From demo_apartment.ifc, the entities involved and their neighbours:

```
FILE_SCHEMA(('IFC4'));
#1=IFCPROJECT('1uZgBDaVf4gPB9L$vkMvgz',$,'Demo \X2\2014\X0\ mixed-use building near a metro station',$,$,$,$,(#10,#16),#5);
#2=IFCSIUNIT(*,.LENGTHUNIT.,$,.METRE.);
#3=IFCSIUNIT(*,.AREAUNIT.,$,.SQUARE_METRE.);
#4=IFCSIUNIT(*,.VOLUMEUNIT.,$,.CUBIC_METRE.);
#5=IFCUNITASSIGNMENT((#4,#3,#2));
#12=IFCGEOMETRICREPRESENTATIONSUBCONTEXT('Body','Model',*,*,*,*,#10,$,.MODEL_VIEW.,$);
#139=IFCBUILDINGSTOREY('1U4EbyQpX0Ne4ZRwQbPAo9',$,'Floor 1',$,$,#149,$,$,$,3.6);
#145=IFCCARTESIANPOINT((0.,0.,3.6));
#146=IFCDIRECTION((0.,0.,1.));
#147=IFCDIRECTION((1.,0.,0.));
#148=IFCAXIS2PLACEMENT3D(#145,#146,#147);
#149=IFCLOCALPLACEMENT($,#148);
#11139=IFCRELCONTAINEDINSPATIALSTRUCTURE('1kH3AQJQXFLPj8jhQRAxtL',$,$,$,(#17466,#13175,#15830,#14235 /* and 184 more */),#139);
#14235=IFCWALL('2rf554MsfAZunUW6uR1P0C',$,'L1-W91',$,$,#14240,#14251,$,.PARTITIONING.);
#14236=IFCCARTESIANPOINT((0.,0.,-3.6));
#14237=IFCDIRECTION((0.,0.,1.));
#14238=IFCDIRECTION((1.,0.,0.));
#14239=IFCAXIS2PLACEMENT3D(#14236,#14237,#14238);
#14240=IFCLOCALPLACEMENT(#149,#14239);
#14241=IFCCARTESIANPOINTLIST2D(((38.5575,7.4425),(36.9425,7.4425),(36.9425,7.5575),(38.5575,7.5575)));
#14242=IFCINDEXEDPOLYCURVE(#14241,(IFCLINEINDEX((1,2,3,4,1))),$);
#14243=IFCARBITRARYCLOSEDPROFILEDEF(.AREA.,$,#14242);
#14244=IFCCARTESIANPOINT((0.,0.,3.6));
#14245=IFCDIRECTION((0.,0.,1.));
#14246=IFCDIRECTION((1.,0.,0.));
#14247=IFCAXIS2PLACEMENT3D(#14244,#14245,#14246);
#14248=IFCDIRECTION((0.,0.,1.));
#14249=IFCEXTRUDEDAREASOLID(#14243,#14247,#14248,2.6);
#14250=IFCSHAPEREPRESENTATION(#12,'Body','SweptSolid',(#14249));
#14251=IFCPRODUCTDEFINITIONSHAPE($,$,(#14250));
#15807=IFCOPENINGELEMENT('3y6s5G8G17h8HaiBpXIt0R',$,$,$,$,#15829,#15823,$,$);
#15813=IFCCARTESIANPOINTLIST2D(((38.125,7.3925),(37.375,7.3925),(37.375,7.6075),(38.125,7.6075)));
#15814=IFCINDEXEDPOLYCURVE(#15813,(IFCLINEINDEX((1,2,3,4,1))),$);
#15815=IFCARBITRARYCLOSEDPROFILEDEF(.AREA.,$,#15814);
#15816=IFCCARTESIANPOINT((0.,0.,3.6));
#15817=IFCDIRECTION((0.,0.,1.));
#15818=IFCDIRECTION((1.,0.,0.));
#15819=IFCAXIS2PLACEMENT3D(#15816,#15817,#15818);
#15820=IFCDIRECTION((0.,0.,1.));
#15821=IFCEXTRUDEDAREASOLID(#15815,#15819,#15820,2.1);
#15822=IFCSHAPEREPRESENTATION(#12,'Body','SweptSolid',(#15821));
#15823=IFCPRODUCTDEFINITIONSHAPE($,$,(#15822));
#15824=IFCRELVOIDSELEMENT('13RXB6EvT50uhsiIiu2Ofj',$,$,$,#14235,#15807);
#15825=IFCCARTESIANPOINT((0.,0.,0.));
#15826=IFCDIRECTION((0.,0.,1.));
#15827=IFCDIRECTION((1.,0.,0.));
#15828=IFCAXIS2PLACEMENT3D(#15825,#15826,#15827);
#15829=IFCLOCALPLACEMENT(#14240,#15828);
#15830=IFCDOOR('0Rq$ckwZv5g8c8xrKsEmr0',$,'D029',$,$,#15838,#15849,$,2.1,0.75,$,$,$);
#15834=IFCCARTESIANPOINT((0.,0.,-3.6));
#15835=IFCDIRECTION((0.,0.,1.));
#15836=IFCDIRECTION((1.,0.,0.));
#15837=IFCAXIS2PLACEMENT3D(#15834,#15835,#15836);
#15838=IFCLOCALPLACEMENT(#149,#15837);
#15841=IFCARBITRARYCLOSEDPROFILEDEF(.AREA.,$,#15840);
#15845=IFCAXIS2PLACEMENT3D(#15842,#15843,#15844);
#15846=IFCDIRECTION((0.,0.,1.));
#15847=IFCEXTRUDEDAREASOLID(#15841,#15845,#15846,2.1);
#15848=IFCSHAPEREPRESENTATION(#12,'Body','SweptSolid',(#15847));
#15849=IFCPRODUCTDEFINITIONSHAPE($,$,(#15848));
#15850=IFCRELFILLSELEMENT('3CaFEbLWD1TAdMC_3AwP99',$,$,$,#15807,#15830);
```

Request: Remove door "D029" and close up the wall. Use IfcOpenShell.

```python
import ifcopenshell
import ifcopenshell.api.feature
import ifcopenshell.api.root
import ifcopenshell.geom
import ifcopenshell.util.shape

model = ifcopenshell.open("demo_apartment.ifc")
settings = ifcopenshell.geom.settings()


def volume(element):
    """Net volume in cubic metres, openings subtracted."""
    shape = ifcopenshell.geom.create_shape(settings, element)
    return ifcopenshell.util.shape.get_volume(shape.geometry)


door = model.by_id(15830)
opening = door.FillsVoids[0].RelatingOpeningElement
wall = opening.VoidsElements[0].RelatingBuildingElement
before = volume(wall)

ifcopenshell.api.root.remove_product(model, product=door)
ifcopenshell.api.feature.remove_feature(model, feature=opening)

after = volume(wall)

print(f"wall volume {before:.3f} -> {after:.3f} m3")

model.write("demo_apartment_updated.ifc")
```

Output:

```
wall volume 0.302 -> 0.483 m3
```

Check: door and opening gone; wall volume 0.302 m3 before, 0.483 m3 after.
